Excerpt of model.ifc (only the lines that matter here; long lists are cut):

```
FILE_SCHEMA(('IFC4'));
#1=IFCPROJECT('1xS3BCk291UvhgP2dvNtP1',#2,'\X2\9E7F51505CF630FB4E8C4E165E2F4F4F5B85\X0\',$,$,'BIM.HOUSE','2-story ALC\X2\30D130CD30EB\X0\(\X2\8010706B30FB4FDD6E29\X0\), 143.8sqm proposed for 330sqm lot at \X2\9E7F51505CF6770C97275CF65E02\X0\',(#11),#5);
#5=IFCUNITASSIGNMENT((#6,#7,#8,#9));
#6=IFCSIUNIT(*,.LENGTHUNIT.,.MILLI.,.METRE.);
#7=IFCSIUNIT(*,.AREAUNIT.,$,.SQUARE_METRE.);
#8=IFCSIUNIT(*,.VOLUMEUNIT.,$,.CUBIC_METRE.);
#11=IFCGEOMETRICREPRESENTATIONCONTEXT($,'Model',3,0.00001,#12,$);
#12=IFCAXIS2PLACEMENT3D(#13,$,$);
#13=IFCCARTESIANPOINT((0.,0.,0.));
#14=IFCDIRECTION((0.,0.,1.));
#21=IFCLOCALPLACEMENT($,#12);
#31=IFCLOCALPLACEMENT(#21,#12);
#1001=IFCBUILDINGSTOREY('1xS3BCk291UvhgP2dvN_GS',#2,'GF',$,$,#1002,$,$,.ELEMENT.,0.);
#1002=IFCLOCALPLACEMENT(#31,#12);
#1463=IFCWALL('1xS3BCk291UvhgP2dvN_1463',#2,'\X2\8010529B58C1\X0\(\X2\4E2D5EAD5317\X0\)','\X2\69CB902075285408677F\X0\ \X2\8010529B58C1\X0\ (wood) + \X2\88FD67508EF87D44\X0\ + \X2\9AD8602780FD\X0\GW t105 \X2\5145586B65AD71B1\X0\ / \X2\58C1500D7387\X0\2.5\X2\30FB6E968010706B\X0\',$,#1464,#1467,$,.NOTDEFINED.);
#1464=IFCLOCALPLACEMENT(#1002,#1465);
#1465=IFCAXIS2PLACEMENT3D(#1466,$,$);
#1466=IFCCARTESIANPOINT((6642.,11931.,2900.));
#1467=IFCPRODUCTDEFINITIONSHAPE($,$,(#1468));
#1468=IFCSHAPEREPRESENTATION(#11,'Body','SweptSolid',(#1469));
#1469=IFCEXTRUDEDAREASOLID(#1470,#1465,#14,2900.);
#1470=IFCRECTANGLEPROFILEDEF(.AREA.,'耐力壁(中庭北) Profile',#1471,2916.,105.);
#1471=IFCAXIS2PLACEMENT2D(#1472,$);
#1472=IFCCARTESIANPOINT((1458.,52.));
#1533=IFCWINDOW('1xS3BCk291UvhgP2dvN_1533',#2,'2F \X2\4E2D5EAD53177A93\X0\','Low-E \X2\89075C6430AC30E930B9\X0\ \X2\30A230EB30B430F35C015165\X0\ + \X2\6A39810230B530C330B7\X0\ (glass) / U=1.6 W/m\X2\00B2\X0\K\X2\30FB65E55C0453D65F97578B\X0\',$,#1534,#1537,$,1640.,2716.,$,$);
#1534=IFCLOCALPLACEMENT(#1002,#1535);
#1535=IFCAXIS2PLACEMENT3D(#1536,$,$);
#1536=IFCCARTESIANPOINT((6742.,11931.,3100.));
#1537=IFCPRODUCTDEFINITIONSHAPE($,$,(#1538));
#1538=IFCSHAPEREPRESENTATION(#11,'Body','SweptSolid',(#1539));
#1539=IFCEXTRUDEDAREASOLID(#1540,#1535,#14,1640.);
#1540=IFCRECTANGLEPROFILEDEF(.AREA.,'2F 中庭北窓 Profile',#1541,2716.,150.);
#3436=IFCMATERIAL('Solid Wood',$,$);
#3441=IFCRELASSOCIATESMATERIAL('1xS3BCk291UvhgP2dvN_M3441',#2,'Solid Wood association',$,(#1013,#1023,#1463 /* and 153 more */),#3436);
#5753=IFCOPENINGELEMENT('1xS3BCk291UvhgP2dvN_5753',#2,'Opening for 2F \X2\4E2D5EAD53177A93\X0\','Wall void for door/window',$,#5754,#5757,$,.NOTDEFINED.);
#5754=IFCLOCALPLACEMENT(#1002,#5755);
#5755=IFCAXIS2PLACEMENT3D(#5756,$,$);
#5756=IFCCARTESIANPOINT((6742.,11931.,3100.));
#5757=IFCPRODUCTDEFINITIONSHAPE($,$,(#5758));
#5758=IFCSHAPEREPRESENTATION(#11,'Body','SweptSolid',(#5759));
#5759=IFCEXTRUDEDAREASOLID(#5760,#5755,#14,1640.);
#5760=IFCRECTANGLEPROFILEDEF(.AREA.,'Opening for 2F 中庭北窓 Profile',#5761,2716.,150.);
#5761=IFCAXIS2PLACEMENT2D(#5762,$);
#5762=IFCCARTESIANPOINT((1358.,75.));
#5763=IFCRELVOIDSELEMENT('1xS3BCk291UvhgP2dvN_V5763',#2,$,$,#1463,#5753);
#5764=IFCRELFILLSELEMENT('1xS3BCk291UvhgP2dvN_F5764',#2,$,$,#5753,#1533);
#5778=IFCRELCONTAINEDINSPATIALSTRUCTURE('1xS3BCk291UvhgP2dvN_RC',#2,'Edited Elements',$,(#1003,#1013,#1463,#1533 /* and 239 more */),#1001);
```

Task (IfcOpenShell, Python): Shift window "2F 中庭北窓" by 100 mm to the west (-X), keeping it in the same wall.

```python
import ifcopenshell
import ifcopenshell.api.geometry
import ifcopenshell.util.placement
import ifcopenshell.util.unit

model = ifcopenshell.open("model.ifc")
unit_scale = ifcopenshell.util.unit.calculate_unit_scale(model)

window = model.by_guid("1xS3BCk291UvhgP2dvN_1533")
opening = window.FillsVoids[0].RelatingOpeningElement
wall = opening.VoidsElements[0].RelatingBuildingElement

wall_matrix = ifcopenshell.util.placement.get_local_placement(wall.ObjectPlacement)
shift = wall_matrix[:3, 0] * -0.1 / unit_scale
before = ifcopenshell.util.placement.get_local_placement(window.ObjectPlacement)[:3, 3].copy()

# The window is not placed relative to its opening, so move both.
for product in (opening, window):
    matrix = ifcopenshell.util.placement.get_local_placement(product.ObjectPlacement)
    matrix[:3, 3] += shift
    ifcopenshell.api.geometry.edit_object_placement(model, product=product, matrix=matrix, is_si=False)

after = ifcopenshell.util.placement.get_local_placement(window.ObjectPlacement)[:3, 3]
print("window moved by", (after - before).round(3) + 0.0)

model.write("model-out.ifc")
```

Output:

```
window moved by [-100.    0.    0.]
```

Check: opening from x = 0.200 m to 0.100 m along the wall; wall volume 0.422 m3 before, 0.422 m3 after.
